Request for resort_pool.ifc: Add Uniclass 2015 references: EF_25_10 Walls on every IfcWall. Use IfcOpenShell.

First a look at what the model holds.

```python
import ifcopenshell

model = ifcopenshell.open("resort_pool.ifc")
print(model.schema)
print("classifications:", [c.Name for c in model.by_type("IfcClassification")])
for ifc_class in ("IfcDoor", "IfcRoof", "IfcStair", "IfcWall", "IfcWindow"):
    print(ifc_class, len(model.by_type(ifc_class)))
```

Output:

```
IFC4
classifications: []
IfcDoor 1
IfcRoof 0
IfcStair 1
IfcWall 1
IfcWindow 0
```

```python
import ifcopenshell
import ifcopenshell.api.classification

model = ifcopenshell.open("resort_pool.ifc")

system = ifcopenshell.api.classification.add_classification(model, classification="Uniclass 2015")

codes = {
    "IfcWall": ("EF_25_10", "Walls"),
}
for ifc_class, (code, name) in codes.items():
    products = model.by_type(ifc_class)
    ifcopenshell.api.classification.add_reference(
        model, products=products, classification=system, identification=code, name=name
    )
    print(code, len(products))

model.write("resort_pool_edited.ifc")
```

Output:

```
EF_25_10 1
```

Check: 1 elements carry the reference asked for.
